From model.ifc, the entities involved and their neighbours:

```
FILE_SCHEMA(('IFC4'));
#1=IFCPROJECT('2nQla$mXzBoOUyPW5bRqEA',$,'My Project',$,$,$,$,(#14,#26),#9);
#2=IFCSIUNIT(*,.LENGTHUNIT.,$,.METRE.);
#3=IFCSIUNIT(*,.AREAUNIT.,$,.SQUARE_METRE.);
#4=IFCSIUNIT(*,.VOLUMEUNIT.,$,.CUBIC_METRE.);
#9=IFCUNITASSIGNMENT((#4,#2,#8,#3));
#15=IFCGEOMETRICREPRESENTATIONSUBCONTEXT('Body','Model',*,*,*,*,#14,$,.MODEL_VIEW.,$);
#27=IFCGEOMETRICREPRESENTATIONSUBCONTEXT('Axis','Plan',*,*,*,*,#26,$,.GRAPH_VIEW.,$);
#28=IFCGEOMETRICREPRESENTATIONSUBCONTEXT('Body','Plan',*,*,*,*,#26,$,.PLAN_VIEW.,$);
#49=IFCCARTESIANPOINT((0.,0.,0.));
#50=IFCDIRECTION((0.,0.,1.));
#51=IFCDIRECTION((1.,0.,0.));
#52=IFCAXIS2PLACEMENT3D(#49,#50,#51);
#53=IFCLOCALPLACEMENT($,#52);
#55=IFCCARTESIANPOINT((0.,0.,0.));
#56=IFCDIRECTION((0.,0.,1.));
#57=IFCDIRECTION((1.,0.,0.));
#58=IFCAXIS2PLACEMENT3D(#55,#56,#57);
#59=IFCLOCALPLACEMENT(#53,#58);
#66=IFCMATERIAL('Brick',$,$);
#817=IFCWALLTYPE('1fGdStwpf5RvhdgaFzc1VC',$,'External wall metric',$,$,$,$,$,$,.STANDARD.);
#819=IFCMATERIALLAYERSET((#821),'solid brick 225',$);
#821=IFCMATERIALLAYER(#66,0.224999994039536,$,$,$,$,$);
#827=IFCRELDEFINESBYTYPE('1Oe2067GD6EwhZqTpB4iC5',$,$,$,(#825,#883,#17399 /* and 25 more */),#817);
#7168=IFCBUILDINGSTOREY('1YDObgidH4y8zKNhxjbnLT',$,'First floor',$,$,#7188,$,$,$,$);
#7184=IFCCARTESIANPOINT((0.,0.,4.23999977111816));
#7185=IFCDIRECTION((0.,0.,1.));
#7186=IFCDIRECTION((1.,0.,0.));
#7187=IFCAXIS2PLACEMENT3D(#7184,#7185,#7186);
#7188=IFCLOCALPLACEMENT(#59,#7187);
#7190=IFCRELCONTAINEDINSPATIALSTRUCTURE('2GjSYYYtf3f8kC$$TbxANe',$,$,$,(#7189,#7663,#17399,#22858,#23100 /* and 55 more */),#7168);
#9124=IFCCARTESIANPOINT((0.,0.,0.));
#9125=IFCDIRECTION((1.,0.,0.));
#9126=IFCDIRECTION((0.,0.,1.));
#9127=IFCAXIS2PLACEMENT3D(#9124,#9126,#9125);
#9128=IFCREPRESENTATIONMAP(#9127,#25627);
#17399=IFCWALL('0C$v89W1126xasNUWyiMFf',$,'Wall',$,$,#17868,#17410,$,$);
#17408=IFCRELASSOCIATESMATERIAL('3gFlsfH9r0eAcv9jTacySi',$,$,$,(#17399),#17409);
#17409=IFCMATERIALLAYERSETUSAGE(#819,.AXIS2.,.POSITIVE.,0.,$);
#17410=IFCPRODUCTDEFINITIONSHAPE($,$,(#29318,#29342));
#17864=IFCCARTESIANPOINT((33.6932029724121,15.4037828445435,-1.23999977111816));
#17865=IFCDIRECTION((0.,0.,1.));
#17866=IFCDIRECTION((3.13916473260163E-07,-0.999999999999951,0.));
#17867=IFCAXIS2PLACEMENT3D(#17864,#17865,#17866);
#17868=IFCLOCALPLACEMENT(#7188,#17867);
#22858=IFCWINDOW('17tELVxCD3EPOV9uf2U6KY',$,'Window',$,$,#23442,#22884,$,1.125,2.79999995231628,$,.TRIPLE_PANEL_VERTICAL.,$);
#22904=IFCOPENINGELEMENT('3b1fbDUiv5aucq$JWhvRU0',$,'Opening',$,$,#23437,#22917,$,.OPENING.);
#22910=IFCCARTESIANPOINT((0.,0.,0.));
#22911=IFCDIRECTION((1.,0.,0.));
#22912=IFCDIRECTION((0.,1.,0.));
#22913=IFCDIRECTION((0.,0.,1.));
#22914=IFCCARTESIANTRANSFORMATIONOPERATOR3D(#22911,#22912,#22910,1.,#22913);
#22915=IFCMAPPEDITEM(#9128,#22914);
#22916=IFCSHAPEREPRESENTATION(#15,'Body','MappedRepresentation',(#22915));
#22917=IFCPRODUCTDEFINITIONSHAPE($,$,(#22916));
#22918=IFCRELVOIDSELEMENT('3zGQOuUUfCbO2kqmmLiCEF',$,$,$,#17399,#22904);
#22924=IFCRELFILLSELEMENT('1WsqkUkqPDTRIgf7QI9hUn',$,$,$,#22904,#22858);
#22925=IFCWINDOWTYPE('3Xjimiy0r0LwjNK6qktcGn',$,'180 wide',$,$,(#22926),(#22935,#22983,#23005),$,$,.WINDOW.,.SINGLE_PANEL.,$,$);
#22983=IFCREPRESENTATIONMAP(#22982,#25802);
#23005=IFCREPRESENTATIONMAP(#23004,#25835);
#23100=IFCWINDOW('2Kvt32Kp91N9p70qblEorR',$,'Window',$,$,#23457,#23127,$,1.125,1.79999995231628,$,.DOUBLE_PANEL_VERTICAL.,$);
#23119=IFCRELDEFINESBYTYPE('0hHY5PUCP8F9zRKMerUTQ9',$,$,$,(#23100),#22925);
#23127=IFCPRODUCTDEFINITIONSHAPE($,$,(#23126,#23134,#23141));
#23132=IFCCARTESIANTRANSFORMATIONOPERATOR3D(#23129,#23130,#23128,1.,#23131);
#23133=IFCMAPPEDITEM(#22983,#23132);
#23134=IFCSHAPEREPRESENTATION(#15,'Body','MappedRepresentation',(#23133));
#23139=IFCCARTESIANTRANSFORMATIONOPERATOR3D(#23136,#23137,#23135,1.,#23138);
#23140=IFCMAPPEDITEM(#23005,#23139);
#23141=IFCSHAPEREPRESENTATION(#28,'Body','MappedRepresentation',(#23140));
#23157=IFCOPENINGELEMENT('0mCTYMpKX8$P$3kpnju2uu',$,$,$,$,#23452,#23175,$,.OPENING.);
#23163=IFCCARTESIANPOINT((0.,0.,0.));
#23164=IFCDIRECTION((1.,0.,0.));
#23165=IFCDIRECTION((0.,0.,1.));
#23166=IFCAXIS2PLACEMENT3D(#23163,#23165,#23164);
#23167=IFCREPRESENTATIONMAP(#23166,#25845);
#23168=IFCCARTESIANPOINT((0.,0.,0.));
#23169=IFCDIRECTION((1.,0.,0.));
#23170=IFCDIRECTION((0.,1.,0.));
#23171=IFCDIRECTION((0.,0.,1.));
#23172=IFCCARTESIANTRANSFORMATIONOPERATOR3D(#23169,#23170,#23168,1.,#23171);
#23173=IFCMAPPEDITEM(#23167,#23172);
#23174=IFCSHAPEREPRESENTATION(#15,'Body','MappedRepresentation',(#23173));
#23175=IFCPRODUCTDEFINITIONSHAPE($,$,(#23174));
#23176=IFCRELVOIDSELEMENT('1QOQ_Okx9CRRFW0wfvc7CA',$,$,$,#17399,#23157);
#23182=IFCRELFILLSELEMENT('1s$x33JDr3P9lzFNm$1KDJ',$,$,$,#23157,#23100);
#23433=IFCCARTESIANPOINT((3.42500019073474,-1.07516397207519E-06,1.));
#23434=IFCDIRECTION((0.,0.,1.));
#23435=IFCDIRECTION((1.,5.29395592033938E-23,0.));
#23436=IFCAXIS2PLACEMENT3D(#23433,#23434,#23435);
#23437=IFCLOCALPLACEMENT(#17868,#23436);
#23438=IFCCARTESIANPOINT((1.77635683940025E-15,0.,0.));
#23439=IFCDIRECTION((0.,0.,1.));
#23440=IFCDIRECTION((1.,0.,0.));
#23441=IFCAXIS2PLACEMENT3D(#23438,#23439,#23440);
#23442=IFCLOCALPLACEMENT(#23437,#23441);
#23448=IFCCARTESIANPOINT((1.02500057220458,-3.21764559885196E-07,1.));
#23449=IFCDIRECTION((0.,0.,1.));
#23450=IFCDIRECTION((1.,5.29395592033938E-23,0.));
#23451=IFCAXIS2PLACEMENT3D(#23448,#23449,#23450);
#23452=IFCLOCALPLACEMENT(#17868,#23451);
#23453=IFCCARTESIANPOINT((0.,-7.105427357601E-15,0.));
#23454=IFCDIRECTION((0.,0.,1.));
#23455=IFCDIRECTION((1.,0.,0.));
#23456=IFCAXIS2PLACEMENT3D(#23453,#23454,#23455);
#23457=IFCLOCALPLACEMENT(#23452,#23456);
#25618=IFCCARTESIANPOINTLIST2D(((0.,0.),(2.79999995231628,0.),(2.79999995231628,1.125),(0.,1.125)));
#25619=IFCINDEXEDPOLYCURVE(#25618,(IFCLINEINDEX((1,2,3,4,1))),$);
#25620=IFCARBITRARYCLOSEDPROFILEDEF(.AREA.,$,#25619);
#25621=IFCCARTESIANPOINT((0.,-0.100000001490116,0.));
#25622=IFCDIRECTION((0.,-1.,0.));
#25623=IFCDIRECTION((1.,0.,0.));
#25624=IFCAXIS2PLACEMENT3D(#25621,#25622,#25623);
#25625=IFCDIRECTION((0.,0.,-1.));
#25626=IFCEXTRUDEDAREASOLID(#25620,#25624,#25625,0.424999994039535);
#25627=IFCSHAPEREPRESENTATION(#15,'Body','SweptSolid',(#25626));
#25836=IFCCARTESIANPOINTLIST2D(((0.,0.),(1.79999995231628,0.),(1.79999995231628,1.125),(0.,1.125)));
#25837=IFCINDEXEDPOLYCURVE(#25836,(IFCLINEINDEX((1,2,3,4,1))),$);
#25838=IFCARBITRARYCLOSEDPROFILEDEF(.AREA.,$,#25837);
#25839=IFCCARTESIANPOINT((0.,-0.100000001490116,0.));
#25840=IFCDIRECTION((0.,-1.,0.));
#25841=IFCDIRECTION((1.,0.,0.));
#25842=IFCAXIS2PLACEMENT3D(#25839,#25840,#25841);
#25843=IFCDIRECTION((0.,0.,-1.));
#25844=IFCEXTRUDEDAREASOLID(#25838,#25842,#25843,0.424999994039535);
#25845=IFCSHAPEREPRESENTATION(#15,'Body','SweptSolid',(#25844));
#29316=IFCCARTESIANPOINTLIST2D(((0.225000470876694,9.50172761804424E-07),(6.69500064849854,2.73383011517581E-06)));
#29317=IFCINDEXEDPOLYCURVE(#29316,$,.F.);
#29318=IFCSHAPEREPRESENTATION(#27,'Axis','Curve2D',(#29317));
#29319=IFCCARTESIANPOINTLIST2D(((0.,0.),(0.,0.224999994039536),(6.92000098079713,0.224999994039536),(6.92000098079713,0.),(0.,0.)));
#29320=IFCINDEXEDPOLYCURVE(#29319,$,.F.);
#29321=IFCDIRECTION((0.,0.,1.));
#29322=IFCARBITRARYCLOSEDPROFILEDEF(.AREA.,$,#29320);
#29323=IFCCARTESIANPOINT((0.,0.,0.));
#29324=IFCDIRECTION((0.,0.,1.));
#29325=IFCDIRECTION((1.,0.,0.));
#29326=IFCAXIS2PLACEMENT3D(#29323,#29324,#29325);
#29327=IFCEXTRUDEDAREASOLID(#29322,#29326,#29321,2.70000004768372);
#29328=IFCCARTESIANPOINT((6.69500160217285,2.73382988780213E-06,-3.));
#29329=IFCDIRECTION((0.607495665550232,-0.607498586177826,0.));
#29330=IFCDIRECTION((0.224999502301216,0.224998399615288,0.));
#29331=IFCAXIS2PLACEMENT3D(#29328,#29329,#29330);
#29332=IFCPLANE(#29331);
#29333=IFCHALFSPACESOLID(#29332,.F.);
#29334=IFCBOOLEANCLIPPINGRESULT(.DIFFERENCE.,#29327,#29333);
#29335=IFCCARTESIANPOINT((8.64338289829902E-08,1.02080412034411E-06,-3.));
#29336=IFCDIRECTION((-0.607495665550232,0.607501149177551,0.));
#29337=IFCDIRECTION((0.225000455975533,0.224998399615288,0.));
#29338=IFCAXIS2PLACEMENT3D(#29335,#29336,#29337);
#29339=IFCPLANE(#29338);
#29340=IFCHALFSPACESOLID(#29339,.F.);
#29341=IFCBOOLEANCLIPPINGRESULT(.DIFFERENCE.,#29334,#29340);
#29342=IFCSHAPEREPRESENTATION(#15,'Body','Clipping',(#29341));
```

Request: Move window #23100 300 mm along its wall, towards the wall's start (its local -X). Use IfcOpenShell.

```python
import ifcopenshell
import ifcopenshell.api.geometry
import ifcopenshell.util.placement
import ifcopenshell.util.unit

model = ifcopenshell.open("model.ifc")
unit_scale = ifcopenshell.util.unit.calculate_unit_scale(model)

window = model.by_guid("2Kvt32Kp91N9p70qblEorR")
opening = window.FillsVoids[0].RelatingOpeningElement
wall = opening.VoidsElements[0].RelatingBuildingElement

wall_matrix = ifcopenshell.util.placement.get_local_placement(wall.ObjectPlacement)
shift = wall_matrix[:3, 0] * -0.3 / unit_scale
before = ifcopenshell.util.placement.get_local_placement(window.ObjectPlacement)[:3, 3].copy()

# The window is placed relative to its opening, so it follows when the opening moves.
matrix = ifcopenshell.util.placement.get_local_placement(opening.ObjectPlacement)
matrix[:3, 3] += shift
ifcopenshell.api.geometry.edit_object_placement(
    model, product=opening, matrix=matrix, is_si=False, should_transform_children=True
)

after = ifcopenshell.util.placement.get_local_placement(window.ObjectPlacement)[:3, 3]
print("window moved by", (after - before).round(3) + 0.0)

model.write("model-out.ifc")
```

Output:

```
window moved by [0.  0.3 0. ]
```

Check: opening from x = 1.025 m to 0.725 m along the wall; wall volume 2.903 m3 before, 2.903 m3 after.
